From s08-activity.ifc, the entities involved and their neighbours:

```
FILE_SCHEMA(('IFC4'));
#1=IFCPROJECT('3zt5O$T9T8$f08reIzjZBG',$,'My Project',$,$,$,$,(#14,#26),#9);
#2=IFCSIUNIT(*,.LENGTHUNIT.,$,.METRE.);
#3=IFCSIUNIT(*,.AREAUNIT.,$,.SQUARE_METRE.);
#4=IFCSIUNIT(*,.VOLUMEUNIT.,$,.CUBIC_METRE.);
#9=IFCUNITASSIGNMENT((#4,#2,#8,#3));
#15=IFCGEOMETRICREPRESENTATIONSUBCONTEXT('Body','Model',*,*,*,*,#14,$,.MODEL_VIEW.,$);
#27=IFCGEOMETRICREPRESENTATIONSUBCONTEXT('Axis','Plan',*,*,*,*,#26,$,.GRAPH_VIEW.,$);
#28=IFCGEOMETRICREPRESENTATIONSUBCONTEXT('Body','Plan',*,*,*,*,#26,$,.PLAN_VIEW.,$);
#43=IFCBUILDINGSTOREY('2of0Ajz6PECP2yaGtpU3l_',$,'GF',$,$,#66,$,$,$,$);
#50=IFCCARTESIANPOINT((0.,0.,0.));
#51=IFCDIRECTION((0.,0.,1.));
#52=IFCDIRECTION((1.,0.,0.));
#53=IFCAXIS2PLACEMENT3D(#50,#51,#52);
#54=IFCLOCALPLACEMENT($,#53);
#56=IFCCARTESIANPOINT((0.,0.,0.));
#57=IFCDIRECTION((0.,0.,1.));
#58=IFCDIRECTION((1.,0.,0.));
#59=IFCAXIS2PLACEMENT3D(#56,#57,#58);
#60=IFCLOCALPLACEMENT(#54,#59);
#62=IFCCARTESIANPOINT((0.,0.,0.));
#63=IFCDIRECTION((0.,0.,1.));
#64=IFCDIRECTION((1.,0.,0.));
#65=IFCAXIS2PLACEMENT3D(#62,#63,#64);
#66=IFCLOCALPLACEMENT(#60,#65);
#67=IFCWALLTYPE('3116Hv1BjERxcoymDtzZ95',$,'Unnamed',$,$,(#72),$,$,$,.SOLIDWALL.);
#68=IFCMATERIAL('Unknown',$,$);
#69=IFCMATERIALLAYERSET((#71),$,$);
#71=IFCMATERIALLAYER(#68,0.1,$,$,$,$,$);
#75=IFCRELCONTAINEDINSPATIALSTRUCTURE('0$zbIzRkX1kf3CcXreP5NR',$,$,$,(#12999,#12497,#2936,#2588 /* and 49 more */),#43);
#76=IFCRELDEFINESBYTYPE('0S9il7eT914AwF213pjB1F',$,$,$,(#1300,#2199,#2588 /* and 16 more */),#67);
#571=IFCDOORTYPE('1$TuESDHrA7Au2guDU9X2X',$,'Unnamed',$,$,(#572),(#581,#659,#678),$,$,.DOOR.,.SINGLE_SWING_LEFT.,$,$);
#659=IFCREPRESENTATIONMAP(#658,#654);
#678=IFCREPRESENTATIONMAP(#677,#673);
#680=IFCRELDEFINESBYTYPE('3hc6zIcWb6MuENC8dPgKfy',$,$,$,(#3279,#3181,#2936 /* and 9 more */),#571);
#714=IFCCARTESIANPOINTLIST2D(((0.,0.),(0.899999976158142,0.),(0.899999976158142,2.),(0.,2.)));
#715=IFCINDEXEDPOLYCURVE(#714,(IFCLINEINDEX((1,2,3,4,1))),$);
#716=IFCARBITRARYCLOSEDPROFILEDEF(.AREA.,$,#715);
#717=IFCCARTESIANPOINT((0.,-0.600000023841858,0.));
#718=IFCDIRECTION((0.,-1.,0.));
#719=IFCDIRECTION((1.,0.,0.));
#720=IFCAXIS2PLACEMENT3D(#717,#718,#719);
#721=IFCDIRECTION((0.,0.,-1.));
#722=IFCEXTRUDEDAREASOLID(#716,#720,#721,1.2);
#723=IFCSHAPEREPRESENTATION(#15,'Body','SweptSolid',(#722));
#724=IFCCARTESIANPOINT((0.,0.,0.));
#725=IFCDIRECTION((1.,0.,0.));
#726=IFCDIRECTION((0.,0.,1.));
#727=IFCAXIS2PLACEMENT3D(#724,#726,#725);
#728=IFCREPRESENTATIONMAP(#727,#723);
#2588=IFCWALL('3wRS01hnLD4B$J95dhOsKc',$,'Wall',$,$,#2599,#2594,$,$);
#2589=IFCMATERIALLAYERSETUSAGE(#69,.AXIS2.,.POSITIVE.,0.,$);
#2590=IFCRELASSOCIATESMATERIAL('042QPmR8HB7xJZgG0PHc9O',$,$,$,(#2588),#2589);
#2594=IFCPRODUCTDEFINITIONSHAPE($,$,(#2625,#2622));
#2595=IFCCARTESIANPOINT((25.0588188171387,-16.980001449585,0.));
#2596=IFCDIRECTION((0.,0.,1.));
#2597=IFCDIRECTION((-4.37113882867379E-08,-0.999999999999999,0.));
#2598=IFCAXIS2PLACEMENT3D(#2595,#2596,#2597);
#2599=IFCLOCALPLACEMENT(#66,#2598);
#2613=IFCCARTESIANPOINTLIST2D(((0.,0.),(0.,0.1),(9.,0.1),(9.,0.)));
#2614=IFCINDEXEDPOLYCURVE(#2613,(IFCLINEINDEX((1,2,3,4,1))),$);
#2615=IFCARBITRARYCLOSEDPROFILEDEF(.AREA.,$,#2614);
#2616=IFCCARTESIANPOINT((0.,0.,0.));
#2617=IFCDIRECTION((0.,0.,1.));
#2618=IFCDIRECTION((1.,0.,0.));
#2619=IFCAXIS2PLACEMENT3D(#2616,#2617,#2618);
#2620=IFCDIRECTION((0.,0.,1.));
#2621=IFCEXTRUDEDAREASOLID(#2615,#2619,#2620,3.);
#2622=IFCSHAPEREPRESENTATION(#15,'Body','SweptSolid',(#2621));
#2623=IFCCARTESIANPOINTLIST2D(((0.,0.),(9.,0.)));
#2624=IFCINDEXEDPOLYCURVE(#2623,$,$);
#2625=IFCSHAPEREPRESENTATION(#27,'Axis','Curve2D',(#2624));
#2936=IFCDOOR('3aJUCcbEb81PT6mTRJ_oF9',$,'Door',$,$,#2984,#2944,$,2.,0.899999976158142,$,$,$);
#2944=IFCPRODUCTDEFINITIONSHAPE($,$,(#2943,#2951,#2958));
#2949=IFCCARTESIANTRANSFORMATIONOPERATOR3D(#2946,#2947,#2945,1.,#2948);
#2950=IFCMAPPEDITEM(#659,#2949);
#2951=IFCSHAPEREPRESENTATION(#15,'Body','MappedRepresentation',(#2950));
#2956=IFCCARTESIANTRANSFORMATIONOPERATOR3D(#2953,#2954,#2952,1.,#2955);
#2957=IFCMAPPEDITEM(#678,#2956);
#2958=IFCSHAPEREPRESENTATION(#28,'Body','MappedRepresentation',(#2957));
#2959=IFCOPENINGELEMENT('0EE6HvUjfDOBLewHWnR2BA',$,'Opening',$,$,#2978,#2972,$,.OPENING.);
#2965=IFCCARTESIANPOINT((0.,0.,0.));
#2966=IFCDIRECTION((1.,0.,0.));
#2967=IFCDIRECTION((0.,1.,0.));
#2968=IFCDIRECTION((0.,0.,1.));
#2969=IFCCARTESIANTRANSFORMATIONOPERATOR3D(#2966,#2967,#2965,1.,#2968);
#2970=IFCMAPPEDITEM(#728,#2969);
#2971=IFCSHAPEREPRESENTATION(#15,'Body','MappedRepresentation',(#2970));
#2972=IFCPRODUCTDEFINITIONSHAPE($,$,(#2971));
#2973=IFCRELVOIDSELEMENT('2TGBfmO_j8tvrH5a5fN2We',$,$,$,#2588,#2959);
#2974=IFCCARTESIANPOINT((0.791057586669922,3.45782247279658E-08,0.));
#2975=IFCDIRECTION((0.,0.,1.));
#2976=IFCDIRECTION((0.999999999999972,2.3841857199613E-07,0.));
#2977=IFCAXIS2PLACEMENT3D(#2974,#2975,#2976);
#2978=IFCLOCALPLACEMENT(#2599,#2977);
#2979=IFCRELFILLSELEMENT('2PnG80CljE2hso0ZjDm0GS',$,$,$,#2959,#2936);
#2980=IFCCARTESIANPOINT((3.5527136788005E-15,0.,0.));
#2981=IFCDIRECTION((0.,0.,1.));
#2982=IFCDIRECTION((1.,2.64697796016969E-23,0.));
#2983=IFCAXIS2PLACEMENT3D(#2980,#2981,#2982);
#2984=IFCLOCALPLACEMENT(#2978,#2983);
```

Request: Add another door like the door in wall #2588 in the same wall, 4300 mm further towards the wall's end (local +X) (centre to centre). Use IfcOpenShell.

```python
import ifcopenshell
import ifcopenshell.api.feature
import ifcopenshell.api.geometry
import ifcopenshell.api.root
import ifcopenshell.geom
import ifcopenshell.util.element
import ifcopenshell.util.placement
import ifcopenshell.util.shape

model = ifcopenshell.open("s08-activity.ifc")
settings = ifcopenshell.geom.settings()


def volume(element):
    """Net volume in cubic metres, openings subtracted."""
    shape = ifcopenshell.geom.create_shape(settings, element)
    return ifcopenshell.util.shape.get_volume(shape.geometry)


door = model.by_guid("3aJUCcbEb81PT6mTRJ_oF9")
opening = door.FillsVoids[0].RelatingOpeningElement
wall = opening.VoidsElements[0].RelatingBuildingElement
before = volume(wall)
shift = ifcopenshell.util.placement.get_local_placement(wall.ObjectPlacement)[:3, 0] * 4.3

# copy_class copies the void relationship, type, container and properties, but no geometry.
new_opening = ifcopenshell.api.root.copy_class(model, product=opening)
new_opening.Representation = ifcopenshell.util.element.copy_deep(
    model, opening.Representation, exclude=["IfcGeometricRepresentationContext", "IfcRepresentationMap"]
)
new_door = ifcopenshell.api.root.copy_class(model, product=door)
new_door.Representation = ifcopenshell.util.element.copy_deep(
    model, door.Representation, exclude=["IfcGeometricRepresentationContext", "IfcRepresentationMap"]
)
ifcopenshell.api.feature.add_filling(model, opening=new_opening, element=new_door)

for old, new in ((opening, new_opening), (door, new_door)):
    matrix = ifcopenshell.util.placement.get_local_placement(old.ObjectPlacement)
    matrix[:3, 3] += shift
    ifcopenshell.api.geometry.edit_object_placement(model, product=new, matrix=matrix, is_si=False)

after = volume(wall)

print(f"wall volume {before:.3f} -> {after:.3f} m3")

model.write("s08-activity_edited.ifc")
```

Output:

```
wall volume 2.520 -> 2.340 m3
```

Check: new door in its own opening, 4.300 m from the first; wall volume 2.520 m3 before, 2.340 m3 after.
